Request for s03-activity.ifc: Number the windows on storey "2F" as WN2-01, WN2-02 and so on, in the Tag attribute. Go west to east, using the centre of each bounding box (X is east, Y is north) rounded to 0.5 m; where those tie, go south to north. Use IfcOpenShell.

First a look at what the model holds.

```python
import ifcopenshell
import ifcopenshell.util.element
import ifcopenshell.util.placement

model = ifcopenshell.open("s03-activity.ifc")
print(model.schema)
storey = next(s for s in model.by_type("IfcBuildingStorey") if s.Name == "2F")
windows = [e for e in ifcopenshell.util.element.get_decomposition(storey) if e.is_a("IfcWindow")]
for e in sorted(windows, key=lambda e: e.id()):
    origin = ifcopenshell.util.placement.get_local_placement(e.ObjectPlacement)[:3, 3]
    print(e.id(), e.Tag, e.Name, origin.round(2) + 0.0, sep=" | ")
```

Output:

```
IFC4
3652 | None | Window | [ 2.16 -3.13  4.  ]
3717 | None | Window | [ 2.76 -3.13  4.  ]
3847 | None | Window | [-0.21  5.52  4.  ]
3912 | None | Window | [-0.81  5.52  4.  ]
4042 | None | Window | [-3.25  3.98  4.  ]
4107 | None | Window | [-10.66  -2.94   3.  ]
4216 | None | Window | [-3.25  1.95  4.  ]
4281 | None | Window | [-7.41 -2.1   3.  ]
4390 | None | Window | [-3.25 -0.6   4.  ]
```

```python
import ifcopenshell
import ifcopenshell.geom
import ifcopenshell.util.element
import ifcopenshell.util.shape

model = ifcopenshell.open("s03-activity.ifc")
settings = ifcopenshell.geom.settings()
settings.set("use-world-coords", True)


def centre(element):
    shape = ifcopenshell.geom.create_shape(settings, element)
    return ifcopenshell.util.shape.get_bbox_centroid(shape.geometry)


storey = next(s for s in model.by_type("IfcBuildingStorey") if s.Name == "2F")
windows = [e for e in ifcopenshell.util.element.get_decomposition(storey) if e.is_a("IfcWindow")]

# Insertion points can sit at a corner or the storey origin, so sort by the geometry (in metres).
centres = {e: centre(e) for e in windows}
windows.sort(key=lambda e: (round(centres[e][0] / 0.5), centres[e][1]))

for i, e in enumerate(windows, start=1):
    number = f"WN2-{i:02d}"
    e.Tag = number
    print(e.id(), number)

model.write("s03-activity-out.ifc")
```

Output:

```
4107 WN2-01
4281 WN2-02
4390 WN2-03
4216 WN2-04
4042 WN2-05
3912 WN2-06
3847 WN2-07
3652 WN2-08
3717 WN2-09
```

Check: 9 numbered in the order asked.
